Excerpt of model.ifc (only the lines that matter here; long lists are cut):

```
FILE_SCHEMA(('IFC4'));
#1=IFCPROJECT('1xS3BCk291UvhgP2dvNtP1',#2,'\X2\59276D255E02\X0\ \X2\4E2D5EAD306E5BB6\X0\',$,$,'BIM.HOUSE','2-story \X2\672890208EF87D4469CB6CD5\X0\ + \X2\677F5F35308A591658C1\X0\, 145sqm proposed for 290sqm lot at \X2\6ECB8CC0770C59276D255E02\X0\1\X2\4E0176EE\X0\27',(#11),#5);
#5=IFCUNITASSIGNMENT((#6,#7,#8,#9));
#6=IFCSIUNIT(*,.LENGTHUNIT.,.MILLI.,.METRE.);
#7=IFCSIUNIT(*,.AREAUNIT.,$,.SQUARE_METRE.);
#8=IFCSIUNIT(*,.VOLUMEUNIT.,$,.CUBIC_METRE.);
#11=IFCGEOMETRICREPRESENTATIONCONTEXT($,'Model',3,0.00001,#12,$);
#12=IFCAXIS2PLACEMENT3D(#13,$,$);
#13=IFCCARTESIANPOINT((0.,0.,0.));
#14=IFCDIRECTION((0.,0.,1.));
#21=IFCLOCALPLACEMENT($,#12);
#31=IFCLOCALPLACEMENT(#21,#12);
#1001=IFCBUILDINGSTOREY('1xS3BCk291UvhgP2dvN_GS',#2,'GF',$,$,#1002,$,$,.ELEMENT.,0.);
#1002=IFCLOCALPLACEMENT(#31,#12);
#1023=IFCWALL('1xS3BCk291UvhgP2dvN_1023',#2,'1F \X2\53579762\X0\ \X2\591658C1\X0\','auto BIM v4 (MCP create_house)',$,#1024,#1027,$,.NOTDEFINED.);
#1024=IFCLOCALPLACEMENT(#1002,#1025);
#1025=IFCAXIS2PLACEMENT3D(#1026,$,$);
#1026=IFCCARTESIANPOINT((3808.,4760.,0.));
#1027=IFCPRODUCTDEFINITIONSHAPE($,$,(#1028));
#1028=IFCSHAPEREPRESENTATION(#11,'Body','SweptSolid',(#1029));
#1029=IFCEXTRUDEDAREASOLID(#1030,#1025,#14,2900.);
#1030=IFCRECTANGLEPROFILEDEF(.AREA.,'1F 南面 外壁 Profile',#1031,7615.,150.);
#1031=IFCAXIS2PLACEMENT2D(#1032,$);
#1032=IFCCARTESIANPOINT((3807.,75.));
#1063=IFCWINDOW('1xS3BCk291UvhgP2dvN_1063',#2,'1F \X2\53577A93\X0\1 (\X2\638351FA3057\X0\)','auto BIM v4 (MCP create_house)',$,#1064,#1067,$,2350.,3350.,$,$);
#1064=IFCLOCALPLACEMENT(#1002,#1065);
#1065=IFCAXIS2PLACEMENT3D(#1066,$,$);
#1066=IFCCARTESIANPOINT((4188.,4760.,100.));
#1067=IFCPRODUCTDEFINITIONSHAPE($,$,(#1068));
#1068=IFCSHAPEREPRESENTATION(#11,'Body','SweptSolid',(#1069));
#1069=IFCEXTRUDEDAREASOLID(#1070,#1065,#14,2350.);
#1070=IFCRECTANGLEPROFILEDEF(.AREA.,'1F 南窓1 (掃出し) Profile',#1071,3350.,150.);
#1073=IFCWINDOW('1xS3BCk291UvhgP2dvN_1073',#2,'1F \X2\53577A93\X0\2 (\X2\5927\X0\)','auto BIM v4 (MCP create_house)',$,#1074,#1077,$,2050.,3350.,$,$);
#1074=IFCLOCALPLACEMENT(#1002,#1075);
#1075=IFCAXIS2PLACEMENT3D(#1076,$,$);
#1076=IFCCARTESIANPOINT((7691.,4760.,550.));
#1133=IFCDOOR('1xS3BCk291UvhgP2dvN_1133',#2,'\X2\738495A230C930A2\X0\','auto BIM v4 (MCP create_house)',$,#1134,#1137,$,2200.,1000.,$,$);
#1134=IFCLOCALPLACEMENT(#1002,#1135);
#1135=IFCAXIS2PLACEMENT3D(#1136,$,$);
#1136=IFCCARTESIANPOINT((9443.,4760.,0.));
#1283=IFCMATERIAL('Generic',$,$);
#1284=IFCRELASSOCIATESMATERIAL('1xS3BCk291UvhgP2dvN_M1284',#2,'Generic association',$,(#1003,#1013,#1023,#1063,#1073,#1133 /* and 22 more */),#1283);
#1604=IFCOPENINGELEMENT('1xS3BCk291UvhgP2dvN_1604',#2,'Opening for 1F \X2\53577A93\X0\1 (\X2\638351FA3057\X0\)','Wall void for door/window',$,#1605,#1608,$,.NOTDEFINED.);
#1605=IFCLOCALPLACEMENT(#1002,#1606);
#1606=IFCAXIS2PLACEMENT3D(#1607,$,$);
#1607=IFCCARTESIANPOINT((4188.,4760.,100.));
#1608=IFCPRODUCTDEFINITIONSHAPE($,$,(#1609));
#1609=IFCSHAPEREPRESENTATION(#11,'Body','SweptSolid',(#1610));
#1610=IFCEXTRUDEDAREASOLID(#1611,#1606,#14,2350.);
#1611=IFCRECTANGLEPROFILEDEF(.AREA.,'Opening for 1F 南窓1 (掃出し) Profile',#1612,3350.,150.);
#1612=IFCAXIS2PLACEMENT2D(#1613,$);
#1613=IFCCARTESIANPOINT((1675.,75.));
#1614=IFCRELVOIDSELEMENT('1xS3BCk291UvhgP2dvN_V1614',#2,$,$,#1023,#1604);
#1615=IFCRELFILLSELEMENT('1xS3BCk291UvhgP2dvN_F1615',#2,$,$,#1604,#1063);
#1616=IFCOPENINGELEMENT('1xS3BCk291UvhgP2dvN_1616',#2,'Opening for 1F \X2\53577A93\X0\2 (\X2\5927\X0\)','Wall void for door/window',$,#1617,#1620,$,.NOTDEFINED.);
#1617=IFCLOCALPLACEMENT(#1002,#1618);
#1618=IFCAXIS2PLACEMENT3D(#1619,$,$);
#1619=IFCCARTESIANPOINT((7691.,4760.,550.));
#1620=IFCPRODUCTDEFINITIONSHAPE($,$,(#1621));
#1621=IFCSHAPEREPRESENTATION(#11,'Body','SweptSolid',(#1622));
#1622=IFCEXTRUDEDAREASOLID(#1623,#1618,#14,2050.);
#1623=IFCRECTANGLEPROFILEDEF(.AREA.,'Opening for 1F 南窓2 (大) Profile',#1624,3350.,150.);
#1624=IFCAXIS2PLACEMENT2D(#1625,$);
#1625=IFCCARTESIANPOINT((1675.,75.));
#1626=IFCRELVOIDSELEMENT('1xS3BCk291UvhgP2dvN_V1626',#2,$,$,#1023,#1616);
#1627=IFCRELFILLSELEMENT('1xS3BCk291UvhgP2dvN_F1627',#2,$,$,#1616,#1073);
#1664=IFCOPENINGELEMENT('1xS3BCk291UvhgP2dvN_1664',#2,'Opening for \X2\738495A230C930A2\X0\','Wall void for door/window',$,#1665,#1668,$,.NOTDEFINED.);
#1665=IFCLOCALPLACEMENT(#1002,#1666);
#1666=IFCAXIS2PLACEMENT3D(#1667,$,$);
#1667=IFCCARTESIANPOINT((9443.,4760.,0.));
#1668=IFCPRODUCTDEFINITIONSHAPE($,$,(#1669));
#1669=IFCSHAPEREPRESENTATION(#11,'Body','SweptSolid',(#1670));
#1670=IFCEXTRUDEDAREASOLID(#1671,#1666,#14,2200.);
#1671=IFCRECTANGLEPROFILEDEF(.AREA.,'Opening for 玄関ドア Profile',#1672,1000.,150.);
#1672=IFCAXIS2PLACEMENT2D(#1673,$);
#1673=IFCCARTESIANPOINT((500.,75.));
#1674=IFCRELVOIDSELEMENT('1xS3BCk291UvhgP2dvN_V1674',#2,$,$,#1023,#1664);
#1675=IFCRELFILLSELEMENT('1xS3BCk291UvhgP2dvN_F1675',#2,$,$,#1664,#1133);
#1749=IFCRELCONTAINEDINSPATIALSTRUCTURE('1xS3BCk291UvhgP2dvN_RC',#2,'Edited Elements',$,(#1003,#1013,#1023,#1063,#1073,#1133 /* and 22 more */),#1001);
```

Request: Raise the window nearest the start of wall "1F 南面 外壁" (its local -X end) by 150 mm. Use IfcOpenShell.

```python
import numpy as np
import ifcopenshell
import ifcopenshell.api.geometry
import ifcopenshell.util.placement
import ifcopenshell.util.unit

model = ifcopenshell.open("model.ifc")
unit_scale = ifcopenshell.util.unit.calculate_unit_scale(model)

window = model.by_guid("1xS3BCk291UvhgP2dvN_1063")
opening = window.FillsVoids[0].RelatingOpeningElement
dz = 150.0

shift = np.array([0.0, 0.0, dz])
# The window is not placed relative to its opening, so move both.
for product in (opening, window):
    matrix = ifcopenshell.util.placement.get_local_placement(product.ObjectPlacement)
    matrix[:3, 3] += shift
    ifcopenshell.api.geometry.edit_object_placement(model, product=product, matrix=matrix, is_si=False)

print(f"moved by {dz * unit_scale:+.3f} m")

model.write("model_edited.ifc")
```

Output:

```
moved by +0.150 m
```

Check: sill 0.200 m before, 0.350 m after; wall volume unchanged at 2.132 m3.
